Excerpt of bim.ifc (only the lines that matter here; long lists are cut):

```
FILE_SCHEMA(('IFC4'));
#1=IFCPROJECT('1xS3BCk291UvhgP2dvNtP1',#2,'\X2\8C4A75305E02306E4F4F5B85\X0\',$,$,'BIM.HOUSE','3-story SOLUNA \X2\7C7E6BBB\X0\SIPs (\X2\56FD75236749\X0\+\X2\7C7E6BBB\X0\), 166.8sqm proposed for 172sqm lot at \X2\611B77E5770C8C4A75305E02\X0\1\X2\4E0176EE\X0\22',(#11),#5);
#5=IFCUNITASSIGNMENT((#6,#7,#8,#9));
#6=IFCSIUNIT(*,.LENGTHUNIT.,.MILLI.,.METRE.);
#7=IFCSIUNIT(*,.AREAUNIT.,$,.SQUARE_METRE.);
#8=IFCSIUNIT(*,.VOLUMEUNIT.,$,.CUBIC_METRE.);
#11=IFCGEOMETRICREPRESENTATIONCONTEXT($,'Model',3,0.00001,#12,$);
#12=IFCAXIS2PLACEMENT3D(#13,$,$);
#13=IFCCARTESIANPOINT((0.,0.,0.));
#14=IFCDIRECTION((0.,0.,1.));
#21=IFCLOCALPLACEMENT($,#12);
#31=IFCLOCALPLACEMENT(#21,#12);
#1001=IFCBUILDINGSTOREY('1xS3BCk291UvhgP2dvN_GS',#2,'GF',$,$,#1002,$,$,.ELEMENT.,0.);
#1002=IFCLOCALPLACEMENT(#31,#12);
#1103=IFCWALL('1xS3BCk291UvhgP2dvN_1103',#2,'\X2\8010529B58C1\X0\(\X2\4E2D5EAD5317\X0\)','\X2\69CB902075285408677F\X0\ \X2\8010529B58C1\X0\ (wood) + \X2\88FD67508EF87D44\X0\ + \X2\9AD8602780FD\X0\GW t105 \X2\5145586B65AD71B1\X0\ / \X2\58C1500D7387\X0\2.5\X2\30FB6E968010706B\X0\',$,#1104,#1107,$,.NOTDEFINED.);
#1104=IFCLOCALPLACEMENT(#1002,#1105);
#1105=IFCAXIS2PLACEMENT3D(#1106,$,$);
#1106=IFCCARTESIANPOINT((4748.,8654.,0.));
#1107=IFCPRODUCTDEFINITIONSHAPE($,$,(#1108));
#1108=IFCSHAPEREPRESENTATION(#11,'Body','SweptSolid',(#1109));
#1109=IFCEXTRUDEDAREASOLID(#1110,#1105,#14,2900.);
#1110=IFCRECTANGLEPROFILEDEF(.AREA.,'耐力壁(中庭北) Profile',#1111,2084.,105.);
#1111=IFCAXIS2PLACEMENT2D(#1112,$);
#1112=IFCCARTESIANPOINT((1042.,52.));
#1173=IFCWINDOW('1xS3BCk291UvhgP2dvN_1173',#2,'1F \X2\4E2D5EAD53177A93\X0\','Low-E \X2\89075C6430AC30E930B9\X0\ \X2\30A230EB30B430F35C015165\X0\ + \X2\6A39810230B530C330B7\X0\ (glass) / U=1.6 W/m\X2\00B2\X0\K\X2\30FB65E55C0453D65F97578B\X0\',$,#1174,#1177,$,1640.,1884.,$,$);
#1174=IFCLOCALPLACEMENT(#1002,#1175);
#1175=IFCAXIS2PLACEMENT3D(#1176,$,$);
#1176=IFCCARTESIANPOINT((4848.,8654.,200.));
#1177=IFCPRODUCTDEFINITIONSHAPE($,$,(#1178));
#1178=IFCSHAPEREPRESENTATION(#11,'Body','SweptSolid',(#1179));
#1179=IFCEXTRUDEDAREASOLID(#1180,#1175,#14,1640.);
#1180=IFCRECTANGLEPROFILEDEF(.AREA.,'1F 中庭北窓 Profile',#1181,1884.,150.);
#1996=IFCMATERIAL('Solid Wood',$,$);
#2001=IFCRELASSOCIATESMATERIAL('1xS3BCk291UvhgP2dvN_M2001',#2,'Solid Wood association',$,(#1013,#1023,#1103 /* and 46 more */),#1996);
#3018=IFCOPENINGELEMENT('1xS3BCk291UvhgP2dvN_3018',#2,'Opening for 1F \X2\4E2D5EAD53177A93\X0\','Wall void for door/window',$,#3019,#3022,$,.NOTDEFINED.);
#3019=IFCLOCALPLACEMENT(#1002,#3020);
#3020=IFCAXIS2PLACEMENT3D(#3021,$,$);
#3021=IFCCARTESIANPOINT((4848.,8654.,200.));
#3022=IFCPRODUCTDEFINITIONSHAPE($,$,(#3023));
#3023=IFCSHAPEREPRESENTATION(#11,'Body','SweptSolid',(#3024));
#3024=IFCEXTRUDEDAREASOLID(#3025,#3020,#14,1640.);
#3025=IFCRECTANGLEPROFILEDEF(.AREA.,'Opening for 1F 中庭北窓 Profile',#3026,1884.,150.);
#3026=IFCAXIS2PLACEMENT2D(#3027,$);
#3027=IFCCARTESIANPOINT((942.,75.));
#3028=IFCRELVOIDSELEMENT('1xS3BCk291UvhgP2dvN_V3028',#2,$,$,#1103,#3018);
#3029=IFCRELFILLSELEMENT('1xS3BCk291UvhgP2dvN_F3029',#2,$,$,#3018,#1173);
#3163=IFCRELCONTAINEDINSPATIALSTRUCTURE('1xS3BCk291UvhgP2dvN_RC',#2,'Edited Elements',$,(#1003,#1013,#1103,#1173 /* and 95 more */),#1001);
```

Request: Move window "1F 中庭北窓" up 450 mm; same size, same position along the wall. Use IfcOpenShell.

```python
import numpy as np
import ifcopenshell
import ifcopenshell.api.geometry
import ifcopenshell.util.placement
import ifcopenshell.util.unit

model = ifcopenshell.open("bim.ifc")
unit_scale = ifcopenshell.util.unit.calculate_unit_scale(model)

window = model.by_guid("1xS3BCk291UvhgP2dvN_1173")
opening = window.FillsVoids[0].RelatingOpeningElement
dz = 0.45 / unit_scale

shift = np.array([0.0, 0.0, dz])
# The window is not placed relative to its opening, so move both.
for product in (opening, window):
    matrix = ifcopenshell.util.placement.get_local_placement(product.ObjectPlacement)
    matrix[:3, 3] += shift
    ifcopenshell.api.geometry.edit_object_placement(model, product=product, matrix=matrix, is_si=False)

print(f"moved by {dz * unit_scale:+.3f} m")

model.write("bim_rev.ifc")
```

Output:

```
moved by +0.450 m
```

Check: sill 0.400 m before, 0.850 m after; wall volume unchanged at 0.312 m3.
